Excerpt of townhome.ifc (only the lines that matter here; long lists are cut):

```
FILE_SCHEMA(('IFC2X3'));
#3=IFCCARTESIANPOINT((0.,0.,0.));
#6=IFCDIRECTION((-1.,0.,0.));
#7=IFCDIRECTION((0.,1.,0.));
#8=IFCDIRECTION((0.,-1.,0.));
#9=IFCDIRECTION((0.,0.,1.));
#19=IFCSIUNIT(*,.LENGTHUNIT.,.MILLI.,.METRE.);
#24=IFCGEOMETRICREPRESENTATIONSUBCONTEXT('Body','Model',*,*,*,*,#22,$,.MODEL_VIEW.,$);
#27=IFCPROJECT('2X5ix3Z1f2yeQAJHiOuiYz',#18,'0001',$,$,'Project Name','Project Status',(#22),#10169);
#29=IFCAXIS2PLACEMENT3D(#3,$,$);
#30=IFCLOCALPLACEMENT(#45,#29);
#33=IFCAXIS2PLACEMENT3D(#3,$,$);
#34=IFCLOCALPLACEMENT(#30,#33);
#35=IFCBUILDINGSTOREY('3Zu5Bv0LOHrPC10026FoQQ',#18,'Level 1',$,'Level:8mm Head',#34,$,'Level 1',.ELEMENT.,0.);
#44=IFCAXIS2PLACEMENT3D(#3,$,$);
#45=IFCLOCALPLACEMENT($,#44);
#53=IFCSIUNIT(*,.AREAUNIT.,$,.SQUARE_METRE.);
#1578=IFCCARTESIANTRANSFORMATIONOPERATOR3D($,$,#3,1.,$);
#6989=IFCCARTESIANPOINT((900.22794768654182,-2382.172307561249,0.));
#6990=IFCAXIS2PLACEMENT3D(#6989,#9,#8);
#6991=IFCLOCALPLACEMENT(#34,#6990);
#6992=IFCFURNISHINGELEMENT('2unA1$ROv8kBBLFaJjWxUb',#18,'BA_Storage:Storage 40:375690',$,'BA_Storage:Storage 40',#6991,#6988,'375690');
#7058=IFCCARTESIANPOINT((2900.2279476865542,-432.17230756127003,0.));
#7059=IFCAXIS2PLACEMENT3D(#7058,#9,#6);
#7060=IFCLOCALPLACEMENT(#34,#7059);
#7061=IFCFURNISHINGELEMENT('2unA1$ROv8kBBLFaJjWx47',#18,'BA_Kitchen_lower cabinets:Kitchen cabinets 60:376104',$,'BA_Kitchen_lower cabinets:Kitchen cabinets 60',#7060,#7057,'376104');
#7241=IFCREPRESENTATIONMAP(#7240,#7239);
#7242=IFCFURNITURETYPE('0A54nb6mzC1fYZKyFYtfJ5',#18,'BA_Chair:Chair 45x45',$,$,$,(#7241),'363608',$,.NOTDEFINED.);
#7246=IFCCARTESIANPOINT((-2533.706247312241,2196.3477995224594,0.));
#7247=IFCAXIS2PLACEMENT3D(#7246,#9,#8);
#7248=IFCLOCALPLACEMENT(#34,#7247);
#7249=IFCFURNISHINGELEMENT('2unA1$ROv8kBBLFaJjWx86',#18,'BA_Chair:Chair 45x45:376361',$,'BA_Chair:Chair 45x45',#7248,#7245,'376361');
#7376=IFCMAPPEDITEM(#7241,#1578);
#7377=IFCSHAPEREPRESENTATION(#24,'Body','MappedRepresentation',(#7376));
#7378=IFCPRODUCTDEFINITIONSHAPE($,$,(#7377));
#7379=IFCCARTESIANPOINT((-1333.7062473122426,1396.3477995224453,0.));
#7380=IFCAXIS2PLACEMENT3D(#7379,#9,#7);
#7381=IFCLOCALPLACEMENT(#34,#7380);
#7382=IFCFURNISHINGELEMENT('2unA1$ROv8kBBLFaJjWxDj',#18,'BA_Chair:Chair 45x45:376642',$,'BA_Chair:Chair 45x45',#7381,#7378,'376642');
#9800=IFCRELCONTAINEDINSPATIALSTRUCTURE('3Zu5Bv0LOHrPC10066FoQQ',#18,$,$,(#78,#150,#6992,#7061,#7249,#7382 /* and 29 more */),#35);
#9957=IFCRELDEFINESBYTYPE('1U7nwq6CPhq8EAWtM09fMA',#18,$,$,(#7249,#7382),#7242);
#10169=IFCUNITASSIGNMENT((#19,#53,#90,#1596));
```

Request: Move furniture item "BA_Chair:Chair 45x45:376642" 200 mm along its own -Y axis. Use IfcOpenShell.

```python
import ifcopenshell
import ifcopenshell.api.geometry
import ifcopenshell.util.placement
import ifcopenshell.util.unit

model = ifcopenshell.open("townhome.ifc")
unit_scale = ifcopenshell.util.unit.calculate_unit_scale(model)

item = model.by_guid("2unA1$ROv8kBBLFaJjWxDj")
matrix = ifcopenshell.util.placement.get_local_placement(item.ObjectPlacement)
matrix[:3, 3] -= matrix[:3, 1] * 0.2 / unit_scale
ifcopenshell.api.geometry.edit_object_placement(model, product=item, matrix=matrix, is_si=False)

print(ifcopenshell.util.placement.get_local_placement(item.ObjectPlacement).round(3) + 0.0)

model.write("townhome-out.ifc")
```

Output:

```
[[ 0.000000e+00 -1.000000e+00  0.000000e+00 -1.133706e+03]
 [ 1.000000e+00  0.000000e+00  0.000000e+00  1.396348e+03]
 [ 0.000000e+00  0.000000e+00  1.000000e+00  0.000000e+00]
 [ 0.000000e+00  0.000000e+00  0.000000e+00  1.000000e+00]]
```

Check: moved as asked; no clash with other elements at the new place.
